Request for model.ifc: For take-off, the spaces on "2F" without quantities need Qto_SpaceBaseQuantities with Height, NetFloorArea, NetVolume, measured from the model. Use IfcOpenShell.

First a look at what the model holds.

```python
import ifcopenshell
import ifcopenshell.util.element
import ifcopenshell.util.unit

model = ifcopenshell.open("model.ifc")
print(model.schema)
for unit_type in ("LENGTHUNIT", "AREAUNIT", "VOLUMEUNIT"):
    print(unit_type, ifcopenshell.util.unit.calculate_unit_scale(model, unit_type))
storey = next(s for s in model.by_type("IfcBuildingStorey") if s.Name == "2F")
spaces = [e for e in ifcopenshell.util.element.get_decomposition(storey) if e.is_a("IfcSpace")]
for e in sorted(spaces, key=lambda e: e.id()):
    print(e.id(), e.is_a(), e.Name, list(ifcopenshell.util.element.get_psets(e, qtos_only=True)), sep=" | ")
```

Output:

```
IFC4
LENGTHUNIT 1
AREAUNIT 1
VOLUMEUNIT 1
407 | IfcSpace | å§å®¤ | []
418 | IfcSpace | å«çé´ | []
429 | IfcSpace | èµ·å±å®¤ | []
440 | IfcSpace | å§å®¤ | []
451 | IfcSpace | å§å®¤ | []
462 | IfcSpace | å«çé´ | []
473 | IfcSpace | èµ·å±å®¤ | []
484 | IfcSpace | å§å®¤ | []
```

```python
import ifcopenshell
import ifcopenshell.api.pset
import ifcopenshell.geom
import ifcopenshell.util.element
import ifcopenshell.util.shape
import ifcopenshell.util.unit

model = ifcopenshell.open("model.ifc")
unit_scale = ifcopenshell.util.unit.calculate_unit_scale(model)
area_scale = ifcopenshell.util.unit.calculate_unit_scale(model, "AREAUNIT")
volume_scale = ifcopenshell.util.unit.calculate_unit_scale(model, "VOLUMEUNIT")
settings = ifcopenshell.geom.settings()

storey = next(s for s in model.by_type("IfcBuildingStorey") if s.Name == "2F")
spaces = [e for e in ifcopenshell.util.element.get_decomposition(storey) if e.is_a("IfcSpace")]

for e in sorted(spaces, key=lambda e: e.id()):
    if ifcopenshell.util.element.get_psets(e, qtos_only=True, should_inherit=False):
        continue
    # Geometry comes back in metres, in the element's own axes.
    shape = ifcopenshell.geom.create_shape(settings, e)
    values = {
        "Height": ifcopenshell.util.shape.get_z(shape.geometry) / unit_scale,
        "NetFloorArea": ifcopenshell.util.shape.get_footprint_area(shape.geometry) / area_scale,
        "NetVolume": ifcopenshell.util.shape.get_volume(shape.geometry) / volume_scale,
    }
    qto = ifcopenshell.api.pset.add_qto(model, product=e, name="Qto_SpaceBaseQuantities")
    ifcopenshell.api.pset.edit_qto(model, qto=qto, properties=values)
    print(e.id(), {k: round(v, 3) for k, v in values.items()})

model.write("model_v2.ifc")
```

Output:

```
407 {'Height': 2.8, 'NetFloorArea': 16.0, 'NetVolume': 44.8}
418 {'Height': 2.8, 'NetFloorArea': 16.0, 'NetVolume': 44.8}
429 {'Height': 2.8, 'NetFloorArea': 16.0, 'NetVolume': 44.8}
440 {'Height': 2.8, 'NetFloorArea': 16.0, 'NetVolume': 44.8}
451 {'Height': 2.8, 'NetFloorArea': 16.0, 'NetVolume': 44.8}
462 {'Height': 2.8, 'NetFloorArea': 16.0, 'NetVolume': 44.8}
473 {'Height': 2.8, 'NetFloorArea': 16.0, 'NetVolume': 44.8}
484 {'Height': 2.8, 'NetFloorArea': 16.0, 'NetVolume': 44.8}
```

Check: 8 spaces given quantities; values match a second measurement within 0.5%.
